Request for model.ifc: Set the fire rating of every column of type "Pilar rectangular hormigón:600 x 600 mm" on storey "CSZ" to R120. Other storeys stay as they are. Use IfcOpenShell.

First a look at what the model holds.

```python
import ifcopenshell
import ifcopenshell.util.element

model = ifcopenshell.open("model.ifc")
print(model.schema)
storey = next(s for s in model.by_type("IfcBuildingStorey") if s.Name == "CSZ")
columns = [e for e in ifcopenshell.util.element.get_decomposition(storey) if e.is_a("IfcColumn")]
seen = {}
for e in columns:
    element_type = ifcopenshell.util.element.get_type(e)
    key = (element_type.Name if element_type != e and element_type else None, ifcopenshell.util.element.get_pset(e, "Pset_ColumnCommon", "FireRating"))
    seen[key] = seen.get(key, 0) + 1
for (name, value), count in sorted(seen.items(), key=str):
    print(count, "x", name, "|", value)
```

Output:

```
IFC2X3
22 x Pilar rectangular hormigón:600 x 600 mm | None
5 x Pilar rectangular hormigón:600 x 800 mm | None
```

```python
import ifcopenshell
import ifcopenshell.api.pset
import ifcopenshell.util.element

model = ifcopenshell.open("model.ifc")

storey = next(s for s in model.by_type("IfcBuildingStorey") if s.Name == "CSZ")
columns = [e for e in ifcopenshell.util.element.get_decomposition(storey) if e.is_a("IfcColumn")]

count = 0
for e in columns:
    element_type = ifcopenshell.util.element.get_type(e)
    if element_type in (None, e) or element_type.Name != "Pilar rectangular hormigón:600 x 600 mm":
        continue
    # add_pset returns the element's existing set when there is one.
    pset = ifcopenshell.api.pset.add_pset(model, product=e, name="Pset_ColumnCommon")
    ifcopenshell.api.pset.edit_pset(model, pset=pset, properties={"FireRating": "R120"})
    count += 1

print(count, "columns updated")

model.write("model_rev.ifc")
```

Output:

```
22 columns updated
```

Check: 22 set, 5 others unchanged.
